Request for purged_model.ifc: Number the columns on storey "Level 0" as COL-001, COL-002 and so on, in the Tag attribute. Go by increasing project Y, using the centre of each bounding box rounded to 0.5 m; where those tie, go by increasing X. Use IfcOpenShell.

First a look at what the model holds.

```python
import ifcopenshell
import ifcopenshell.util.element
import ifcopenshell.util.placement

model = ifcopenshell.open("purged_model.ifc")
print(model.schema)
storey = next(s for s in model.by_type("IfcBuildingStorey") if s.Name == "Level 0")
columns = [e for e in ifcopenshell.util.element.get_decomposition(storey) if e.is_a("IfcColumn")]
for e in sorted(columns, key=lambda e: e.id()):
    origin = ifcopenshell.util.placement.get_local_placement(e.ObjectPlacement)[:3, 3]
    print(e.id(), e.Tag, e.Name, origin.round(2) + 0.0, sep=" | ")
```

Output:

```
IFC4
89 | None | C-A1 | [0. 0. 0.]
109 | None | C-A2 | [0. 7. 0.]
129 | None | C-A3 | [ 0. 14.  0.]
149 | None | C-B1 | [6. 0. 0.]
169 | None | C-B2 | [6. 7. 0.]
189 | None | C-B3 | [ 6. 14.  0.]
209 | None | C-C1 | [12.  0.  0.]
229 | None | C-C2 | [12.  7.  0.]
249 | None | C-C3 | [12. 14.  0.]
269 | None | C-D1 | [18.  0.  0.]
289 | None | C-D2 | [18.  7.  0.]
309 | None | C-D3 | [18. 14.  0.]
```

```python
import ifcopenshell
import ifcopenshell.geom
import ifcopenshell.util.element
import ifcopenshell.util.shape

model = ifcopenshell.open("purged_model.ifc")
settings = ifcopenshell.geom.settings()
settings.set("use-world-coords", True)


def centre(element):
    shape = ifcopenshell.geom.create_shape(settings, element)
    return ifcopenshell.util.shape.get_bbox_centroid(shape.geometry)


storey = next(s for s in model.by_type("IfcBuildingStorey") if s.Name == "Level 0")
columns = [e for e in ifcopenshell.util.element.get_decomposition(storey) if e.is_a("IfcColumn")]

# Insertion points can sit at a corner or the storey origin, so sort by the geometry (in metres).
centres = {e: centre(e) for e in columns}
columns.sort(key=lambda e: (round(centres[e][1] / 0.5), centres[e][0]))

for i, e in enumerate(columns, start=1):
    number = f"COL-0{i:02d}"
    e.Tag = number
    print(e.id(), number)

model.write("purged_model_v2.ifc")
```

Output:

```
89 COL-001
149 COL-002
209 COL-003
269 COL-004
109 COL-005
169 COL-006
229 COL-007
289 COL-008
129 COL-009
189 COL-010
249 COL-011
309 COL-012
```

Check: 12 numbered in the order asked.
